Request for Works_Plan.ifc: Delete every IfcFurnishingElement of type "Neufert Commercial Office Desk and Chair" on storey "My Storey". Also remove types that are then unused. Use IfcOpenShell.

First a look at what the model holds.

```python
import ifcopenshell
import ifcopenshell.util.element

model = ifcopenshell.open("Works_Plan.ifc")
print(model.schema)
storey = next(s for s in model.by_type("IfcBuildingStorey") if s.Name == "My Storey")
furniture = [e for e in ifcopenshell.util.element.get_decomposition(storey) if e.is_a("IfcFurnishingElement")]
seen = {}
for e in furniture:
    element_type = ifcopenshell.util.element.get_type(e)
    name = element_type.Name if element_type not in (None, e) else None
    seen[name] = seen.get(name, 0) + 1
for name, count in sorted(seen.items(), key=str):
    print(count, "x", name)
```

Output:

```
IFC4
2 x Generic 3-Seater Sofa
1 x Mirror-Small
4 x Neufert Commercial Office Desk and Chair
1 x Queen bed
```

```python
import ifcopenshell
import ifcopenshell.api.root
import ifcopenshell.util.element

model = ifcopenshell.open("Works_Plan.ifc")

storey = next(s for s in model.by_type("IfcBuildingStorey") if s.Name == "My Storey")
furniture = [e for e in ifcopenshell.util.element.get_decomposition(storey) if e.is_a("IfcFurnishingElement")]
targets = [e for e in furniture if (t := ifcopenshell.util.element.get_type(e)) not in (None, e) and t.Name == "Neufert Commercial Office Desk and Chair"]
types = {ifcopenshell.util.element.get_type(e) for e in targets} - {None, *targets}

for e in targets:
    ifcopenshell.api.root.remove_product(model, product=e)
print(len(targets), "removed")

unused = [t for t in types if not ifcopenshell.util.element.get_types(t)]
for t in unused:
    ifcopenshell.api.root.remove_product(model, product=t)
print(len(unused), "unused types removed")

model.write("Works_Plan_edited.ifc")
```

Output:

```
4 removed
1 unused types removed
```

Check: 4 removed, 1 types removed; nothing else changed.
